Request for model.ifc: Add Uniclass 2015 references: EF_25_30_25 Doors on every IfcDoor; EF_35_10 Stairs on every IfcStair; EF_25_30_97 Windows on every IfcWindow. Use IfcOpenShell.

First a look at what the model holds.

```python
import ifcopenshell

model = ifcopenshell.open("model.ifc")
print(model.schema)
print("classifications:", [c.Name for c in model.by_type("IfcClassification")])
for ifc_class in ("IfcDoor", "IfcRoof", "IfcStair", "IfcWall", "IfcWindow"):
    print(ifc_class, len(model.by_type(ifc_class)))
```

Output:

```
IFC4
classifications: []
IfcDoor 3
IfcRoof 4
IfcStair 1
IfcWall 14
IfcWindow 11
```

```python
import ifcopenshell
import ifcopenshell.api.classification

model = ifcopenshell.open("model.ifc")

system = ifcopenshell.api.classification.add_classification(model, classification="Uniclass 2015")

codes = {
    "IfcDoor": ("EF_25_30_25", "Doors"),
    "IfcStair": ("EF_35_10", "Stairs"),
    "IfcWindow": ("EF_25_30_97", "Windows"),
}
for ifc_class, (code, name) in codes.items():
    products = model.by_type(ifc_class)
    ifcopenshell.api.classification.add_reference(
        model, products=products, classification=system, identification=code, name=name
    )
    print(code, len(products))

model.write("model_edited.ifc")
```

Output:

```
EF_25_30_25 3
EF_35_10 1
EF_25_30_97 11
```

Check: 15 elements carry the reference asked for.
